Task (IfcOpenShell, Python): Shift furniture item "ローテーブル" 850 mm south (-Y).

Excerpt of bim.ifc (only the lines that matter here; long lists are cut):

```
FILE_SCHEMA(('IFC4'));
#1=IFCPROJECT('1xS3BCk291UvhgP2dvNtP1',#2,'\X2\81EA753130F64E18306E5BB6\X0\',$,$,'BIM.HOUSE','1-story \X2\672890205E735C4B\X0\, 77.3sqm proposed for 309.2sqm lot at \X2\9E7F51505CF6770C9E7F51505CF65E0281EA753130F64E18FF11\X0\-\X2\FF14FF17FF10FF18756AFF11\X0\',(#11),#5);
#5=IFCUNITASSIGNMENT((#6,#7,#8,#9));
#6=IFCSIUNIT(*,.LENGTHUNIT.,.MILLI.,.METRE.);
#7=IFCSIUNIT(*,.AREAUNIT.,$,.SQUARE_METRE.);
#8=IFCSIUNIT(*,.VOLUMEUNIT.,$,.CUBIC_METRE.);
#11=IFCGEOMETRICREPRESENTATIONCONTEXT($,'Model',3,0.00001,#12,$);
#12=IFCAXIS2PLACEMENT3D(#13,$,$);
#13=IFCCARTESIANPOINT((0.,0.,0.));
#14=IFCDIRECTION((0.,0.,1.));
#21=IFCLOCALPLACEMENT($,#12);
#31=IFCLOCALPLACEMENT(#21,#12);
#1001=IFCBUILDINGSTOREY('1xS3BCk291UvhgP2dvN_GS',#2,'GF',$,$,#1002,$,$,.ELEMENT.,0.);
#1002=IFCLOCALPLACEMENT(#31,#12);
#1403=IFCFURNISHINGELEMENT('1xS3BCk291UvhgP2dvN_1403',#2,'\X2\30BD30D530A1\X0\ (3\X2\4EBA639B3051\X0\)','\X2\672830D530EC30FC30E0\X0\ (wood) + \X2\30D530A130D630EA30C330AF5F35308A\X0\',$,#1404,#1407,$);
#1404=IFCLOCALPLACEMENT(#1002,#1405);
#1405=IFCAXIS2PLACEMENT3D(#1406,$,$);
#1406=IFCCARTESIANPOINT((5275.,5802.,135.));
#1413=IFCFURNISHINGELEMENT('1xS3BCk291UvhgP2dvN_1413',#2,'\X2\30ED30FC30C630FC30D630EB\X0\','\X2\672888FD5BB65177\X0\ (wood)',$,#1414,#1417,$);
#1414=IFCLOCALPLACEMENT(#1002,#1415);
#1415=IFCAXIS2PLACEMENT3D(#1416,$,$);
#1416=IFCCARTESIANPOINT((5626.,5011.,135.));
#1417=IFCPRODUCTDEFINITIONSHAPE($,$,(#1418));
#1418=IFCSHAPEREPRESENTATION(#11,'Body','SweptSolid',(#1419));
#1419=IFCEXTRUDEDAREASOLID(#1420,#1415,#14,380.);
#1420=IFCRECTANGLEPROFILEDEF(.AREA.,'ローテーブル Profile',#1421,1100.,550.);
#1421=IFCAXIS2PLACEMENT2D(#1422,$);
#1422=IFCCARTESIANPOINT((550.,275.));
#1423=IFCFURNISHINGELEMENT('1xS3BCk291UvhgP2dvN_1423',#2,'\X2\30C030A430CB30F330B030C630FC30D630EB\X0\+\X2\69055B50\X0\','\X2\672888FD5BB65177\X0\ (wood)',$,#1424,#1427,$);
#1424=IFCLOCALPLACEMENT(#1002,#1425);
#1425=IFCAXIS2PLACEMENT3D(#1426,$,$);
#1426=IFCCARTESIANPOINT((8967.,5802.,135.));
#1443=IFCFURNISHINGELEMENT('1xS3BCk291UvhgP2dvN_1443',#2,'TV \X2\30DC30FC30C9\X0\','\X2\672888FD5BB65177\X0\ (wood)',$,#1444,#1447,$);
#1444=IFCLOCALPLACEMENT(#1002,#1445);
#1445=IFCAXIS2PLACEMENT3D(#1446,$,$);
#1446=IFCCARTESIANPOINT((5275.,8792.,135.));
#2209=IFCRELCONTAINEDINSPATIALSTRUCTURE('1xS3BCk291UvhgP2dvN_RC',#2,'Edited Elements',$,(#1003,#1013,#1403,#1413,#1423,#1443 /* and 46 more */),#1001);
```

```python
import ifcopenshell
import ifcopenshell.api.geometry
import ifcopenshell.util.placement
import ifcopenshell.util.unit

model = ifcopenshell.open("bim.ifc")
unit_scale = ifcopenshell.util.unit.calculate_unit_scale(model)

item = model.by_guid("1xS3BCk291UvhgP2dvN_1413")
matrix = ifcopenshell.util.placement.get_local_placement(item.ObjectPlacement)
matrix[1, 3] -= 0.85 / unit_scale
ifcopenshell.api.geometry.edit_object_placement(model, product=item, matrix=matrix, is_si=False)

print(ifcopenshell.util.placement.get_local_placement(item.ObjectPlacement).round(3) + 0.0)

model.write("bim_v2.ifc")
```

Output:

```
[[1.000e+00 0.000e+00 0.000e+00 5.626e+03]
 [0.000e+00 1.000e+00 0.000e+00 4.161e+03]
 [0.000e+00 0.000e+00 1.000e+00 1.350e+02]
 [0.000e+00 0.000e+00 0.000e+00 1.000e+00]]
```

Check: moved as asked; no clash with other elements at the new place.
